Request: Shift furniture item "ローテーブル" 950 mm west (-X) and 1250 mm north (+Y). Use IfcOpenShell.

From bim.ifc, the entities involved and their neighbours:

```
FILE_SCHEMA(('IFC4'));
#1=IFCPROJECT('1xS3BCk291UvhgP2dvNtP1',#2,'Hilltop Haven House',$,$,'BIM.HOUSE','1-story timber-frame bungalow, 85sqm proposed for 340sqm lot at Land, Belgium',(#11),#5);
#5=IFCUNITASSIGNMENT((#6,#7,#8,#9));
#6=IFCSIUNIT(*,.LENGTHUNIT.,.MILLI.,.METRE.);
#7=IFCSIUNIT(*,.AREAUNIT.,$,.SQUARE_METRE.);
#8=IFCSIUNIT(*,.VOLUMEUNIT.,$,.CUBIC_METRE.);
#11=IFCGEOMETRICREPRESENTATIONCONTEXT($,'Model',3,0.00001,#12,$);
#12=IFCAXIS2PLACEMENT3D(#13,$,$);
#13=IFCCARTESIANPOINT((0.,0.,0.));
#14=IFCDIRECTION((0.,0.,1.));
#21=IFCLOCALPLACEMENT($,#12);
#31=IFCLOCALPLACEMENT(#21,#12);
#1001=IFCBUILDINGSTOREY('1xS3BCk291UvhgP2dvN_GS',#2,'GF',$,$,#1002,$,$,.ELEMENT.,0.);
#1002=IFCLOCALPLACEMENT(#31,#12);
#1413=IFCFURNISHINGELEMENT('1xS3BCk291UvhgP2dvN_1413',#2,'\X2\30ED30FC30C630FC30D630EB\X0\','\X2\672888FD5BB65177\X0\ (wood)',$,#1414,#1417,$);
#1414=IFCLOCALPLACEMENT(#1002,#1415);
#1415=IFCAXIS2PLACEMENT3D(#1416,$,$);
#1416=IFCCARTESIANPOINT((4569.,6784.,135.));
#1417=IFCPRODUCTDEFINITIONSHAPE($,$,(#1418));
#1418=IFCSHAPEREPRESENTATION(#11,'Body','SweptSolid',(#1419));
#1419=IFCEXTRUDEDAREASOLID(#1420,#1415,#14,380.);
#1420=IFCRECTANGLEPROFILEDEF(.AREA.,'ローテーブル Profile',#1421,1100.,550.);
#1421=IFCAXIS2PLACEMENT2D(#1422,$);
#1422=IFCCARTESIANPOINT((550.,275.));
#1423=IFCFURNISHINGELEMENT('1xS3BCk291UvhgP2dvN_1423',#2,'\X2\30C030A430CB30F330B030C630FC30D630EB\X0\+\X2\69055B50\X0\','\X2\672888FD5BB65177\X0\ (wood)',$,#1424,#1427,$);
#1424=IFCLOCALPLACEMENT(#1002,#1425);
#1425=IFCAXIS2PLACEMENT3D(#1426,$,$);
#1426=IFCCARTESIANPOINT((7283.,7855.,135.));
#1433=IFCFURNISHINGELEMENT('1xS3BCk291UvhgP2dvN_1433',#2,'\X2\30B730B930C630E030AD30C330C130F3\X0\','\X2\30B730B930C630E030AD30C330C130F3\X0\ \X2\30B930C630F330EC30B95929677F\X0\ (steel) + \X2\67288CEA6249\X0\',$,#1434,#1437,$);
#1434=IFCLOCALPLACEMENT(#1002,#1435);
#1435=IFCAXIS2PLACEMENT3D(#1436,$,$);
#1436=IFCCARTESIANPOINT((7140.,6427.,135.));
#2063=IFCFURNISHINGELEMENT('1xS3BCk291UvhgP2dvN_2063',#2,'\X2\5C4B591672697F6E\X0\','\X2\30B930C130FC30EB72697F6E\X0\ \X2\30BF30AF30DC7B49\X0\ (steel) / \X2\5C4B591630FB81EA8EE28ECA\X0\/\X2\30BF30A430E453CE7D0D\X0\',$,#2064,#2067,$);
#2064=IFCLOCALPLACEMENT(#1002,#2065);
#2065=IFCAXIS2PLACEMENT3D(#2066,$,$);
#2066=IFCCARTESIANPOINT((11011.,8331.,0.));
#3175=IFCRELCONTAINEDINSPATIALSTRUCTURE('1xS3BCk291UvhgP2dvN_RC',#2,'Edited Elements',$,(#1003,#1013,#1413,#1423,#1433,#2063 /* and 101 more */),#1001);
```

```python
import ifcopenshell
import ifcopenshell.api.geometry
import ifcopenshell.util.placement
import ifcopenshell.util.unit

model = ifcopenshell.open("bim.ifc")
unit_scale = ifcopenshell.util.unit.calculate_unit_scale(model)

item = model.by_guid("1xS3BCk291UvhgP2dvN_1413")
matrix = ifcopenshell.util.placement.get_local_placement(item.ObjectPlacement)
matrix[0, 3] -= 0.95 / unit_scale
matrix[1, 3] += 1.25 / unit_scale
ifcopenshell.api.geometry.edit_object_placement(model, product=item, matrix=matrix, is_si=False)

print(ifcopenshell.util.placement.get_local_placement(item.ObjectPlacement).round(3) + 0.0)

model.write("bim-out.ifc")
```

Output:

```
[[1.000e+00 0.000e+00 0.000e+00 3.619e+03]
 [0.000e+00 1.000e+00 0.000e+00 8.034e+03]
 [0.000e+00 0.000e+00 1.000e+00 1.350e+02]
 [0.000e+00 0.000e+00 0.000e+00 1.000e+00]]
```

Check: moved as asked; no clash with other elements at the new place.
